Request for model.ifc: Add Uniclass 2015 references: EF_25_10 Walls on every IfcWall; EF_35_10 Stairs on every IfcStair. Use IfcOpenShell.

First a look at what the model holds.

```python
import ifcopenshell

model = ifcopenshell.open("model.ifc")
print(model.schema)
print("classifications:", [c.Name for c in model.by_type("IfcClassification")])
for ifc_class in ("IfcDoor", "IfcRoof", "IfcStair", "IfcWall", "IfcWindow"):
    print(ifc_class, len(model.by_type(ifc_class)))
```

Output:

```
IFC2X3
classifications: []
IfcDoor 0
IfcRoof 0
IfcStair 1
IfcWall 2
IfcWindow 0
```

```python
import ifcopenshell
import ifcopenshell.api.classification

model = ifcopenshell.open("model.ifc")

# IFC2X3 requires Source and Edition and has no link from the project to the system.
system = model.create_entity("IfcClassification", Source="NBS", Edition="2015", Name="Uniclass 2015")

codes = {
    "IfcWall": ("EF_25_10", "Walls"),
    "IfcStair": ("EF_35_10", "Stairs"),
}
for ifc_class, (code, name) in codes.items():
    products = model.by_type(ifc_class)
    ifcopenshell.api.classification.add_reference(
        model, products=products, classification=system, identification=code, name=name
    )
    print(code, len(products))

model.write("model-out.ifc")
```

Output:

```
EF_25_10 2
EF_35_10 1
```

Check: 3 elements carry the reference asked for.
